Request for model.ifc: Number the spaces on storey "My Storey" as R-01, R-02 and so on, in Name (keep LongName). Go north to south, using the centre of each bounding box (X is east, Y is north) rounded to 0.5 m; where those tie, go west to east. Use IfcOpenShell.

First a look at what the model holds.

```python
import ifcopenshell
import ifcopenshell.util.element
import ifcopenshell.util.placement

model = ifcopenshell.open("model.ifc")
print(model.schema)
storey = next(s for s in model.by_type("IfcBuildingStorey") if s.Name == "My Storey")
spaces = [e for e in ifcopenshell.util.element.get_decomposition(storey) if e.is_a("IfcSpace")]
for e in sorted(spaces, key=lambda e: e.id()):
    origin = ifcopenshell.util.placement.get_local_placement(e.ObjectPlacement)[:3, 3]
    print(e.id(), e.Name, e.LongName, origin.round(2) + 0.0, sep=" | ")
```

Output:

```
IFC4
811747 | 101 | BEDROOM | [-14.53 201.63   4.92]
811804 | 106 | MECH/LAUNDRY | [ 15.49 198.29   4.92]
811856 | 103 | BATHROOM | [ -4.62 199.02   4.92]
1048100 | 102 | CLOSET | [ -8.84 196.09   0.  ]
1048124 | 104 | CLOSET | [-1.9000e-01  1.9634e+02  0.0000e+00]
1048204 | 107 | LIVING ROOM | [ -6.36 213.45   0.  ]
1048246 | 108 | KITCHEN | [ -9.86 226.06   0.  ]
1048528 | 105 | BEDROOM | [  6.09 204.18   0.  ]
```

```python
import ifcopenshell
import ifcopenshell.geom
import ifcopenshell.util.element
import ifcopenshell.util.shape

model = ifcopenshell.open("model.ifc")
settings = ifcopenshell.geom.settings()
settings.set("use-world-coords", True)


def centre(element):
    shape = ifcopenshell.geom.create_shape(settings, element)
    return ifcopenshell.util.shape.get_bbox_centroid(shape.geometry)


storey = next(s for s in model.by_type("IfcBuildingStorey") if s.Name == "My Storey")
spaces = [e for e in ifcopenshell.util.element.get_decomposition(storey) if e.is_a("IfcSpace")]

# Insertion points can sit at a corner or the storey origin, so sort by the geometry (in metres).
centres = {e: centre(e) for e in spaces}
spaces.sort(key=lambda e: (-round(centres[e][1] / 0.5), centres[e][0]))

for i, e in enumerate(spaces, start=1):
    number = f"R-{i:02d}"
    e.Name = number
    print(e.id(), number)

model.write("model_edited.ifc")
```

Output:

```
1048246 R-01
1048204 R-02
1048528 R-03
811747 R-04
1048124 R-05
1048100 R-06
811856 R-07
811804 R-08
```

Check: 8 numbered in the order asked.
